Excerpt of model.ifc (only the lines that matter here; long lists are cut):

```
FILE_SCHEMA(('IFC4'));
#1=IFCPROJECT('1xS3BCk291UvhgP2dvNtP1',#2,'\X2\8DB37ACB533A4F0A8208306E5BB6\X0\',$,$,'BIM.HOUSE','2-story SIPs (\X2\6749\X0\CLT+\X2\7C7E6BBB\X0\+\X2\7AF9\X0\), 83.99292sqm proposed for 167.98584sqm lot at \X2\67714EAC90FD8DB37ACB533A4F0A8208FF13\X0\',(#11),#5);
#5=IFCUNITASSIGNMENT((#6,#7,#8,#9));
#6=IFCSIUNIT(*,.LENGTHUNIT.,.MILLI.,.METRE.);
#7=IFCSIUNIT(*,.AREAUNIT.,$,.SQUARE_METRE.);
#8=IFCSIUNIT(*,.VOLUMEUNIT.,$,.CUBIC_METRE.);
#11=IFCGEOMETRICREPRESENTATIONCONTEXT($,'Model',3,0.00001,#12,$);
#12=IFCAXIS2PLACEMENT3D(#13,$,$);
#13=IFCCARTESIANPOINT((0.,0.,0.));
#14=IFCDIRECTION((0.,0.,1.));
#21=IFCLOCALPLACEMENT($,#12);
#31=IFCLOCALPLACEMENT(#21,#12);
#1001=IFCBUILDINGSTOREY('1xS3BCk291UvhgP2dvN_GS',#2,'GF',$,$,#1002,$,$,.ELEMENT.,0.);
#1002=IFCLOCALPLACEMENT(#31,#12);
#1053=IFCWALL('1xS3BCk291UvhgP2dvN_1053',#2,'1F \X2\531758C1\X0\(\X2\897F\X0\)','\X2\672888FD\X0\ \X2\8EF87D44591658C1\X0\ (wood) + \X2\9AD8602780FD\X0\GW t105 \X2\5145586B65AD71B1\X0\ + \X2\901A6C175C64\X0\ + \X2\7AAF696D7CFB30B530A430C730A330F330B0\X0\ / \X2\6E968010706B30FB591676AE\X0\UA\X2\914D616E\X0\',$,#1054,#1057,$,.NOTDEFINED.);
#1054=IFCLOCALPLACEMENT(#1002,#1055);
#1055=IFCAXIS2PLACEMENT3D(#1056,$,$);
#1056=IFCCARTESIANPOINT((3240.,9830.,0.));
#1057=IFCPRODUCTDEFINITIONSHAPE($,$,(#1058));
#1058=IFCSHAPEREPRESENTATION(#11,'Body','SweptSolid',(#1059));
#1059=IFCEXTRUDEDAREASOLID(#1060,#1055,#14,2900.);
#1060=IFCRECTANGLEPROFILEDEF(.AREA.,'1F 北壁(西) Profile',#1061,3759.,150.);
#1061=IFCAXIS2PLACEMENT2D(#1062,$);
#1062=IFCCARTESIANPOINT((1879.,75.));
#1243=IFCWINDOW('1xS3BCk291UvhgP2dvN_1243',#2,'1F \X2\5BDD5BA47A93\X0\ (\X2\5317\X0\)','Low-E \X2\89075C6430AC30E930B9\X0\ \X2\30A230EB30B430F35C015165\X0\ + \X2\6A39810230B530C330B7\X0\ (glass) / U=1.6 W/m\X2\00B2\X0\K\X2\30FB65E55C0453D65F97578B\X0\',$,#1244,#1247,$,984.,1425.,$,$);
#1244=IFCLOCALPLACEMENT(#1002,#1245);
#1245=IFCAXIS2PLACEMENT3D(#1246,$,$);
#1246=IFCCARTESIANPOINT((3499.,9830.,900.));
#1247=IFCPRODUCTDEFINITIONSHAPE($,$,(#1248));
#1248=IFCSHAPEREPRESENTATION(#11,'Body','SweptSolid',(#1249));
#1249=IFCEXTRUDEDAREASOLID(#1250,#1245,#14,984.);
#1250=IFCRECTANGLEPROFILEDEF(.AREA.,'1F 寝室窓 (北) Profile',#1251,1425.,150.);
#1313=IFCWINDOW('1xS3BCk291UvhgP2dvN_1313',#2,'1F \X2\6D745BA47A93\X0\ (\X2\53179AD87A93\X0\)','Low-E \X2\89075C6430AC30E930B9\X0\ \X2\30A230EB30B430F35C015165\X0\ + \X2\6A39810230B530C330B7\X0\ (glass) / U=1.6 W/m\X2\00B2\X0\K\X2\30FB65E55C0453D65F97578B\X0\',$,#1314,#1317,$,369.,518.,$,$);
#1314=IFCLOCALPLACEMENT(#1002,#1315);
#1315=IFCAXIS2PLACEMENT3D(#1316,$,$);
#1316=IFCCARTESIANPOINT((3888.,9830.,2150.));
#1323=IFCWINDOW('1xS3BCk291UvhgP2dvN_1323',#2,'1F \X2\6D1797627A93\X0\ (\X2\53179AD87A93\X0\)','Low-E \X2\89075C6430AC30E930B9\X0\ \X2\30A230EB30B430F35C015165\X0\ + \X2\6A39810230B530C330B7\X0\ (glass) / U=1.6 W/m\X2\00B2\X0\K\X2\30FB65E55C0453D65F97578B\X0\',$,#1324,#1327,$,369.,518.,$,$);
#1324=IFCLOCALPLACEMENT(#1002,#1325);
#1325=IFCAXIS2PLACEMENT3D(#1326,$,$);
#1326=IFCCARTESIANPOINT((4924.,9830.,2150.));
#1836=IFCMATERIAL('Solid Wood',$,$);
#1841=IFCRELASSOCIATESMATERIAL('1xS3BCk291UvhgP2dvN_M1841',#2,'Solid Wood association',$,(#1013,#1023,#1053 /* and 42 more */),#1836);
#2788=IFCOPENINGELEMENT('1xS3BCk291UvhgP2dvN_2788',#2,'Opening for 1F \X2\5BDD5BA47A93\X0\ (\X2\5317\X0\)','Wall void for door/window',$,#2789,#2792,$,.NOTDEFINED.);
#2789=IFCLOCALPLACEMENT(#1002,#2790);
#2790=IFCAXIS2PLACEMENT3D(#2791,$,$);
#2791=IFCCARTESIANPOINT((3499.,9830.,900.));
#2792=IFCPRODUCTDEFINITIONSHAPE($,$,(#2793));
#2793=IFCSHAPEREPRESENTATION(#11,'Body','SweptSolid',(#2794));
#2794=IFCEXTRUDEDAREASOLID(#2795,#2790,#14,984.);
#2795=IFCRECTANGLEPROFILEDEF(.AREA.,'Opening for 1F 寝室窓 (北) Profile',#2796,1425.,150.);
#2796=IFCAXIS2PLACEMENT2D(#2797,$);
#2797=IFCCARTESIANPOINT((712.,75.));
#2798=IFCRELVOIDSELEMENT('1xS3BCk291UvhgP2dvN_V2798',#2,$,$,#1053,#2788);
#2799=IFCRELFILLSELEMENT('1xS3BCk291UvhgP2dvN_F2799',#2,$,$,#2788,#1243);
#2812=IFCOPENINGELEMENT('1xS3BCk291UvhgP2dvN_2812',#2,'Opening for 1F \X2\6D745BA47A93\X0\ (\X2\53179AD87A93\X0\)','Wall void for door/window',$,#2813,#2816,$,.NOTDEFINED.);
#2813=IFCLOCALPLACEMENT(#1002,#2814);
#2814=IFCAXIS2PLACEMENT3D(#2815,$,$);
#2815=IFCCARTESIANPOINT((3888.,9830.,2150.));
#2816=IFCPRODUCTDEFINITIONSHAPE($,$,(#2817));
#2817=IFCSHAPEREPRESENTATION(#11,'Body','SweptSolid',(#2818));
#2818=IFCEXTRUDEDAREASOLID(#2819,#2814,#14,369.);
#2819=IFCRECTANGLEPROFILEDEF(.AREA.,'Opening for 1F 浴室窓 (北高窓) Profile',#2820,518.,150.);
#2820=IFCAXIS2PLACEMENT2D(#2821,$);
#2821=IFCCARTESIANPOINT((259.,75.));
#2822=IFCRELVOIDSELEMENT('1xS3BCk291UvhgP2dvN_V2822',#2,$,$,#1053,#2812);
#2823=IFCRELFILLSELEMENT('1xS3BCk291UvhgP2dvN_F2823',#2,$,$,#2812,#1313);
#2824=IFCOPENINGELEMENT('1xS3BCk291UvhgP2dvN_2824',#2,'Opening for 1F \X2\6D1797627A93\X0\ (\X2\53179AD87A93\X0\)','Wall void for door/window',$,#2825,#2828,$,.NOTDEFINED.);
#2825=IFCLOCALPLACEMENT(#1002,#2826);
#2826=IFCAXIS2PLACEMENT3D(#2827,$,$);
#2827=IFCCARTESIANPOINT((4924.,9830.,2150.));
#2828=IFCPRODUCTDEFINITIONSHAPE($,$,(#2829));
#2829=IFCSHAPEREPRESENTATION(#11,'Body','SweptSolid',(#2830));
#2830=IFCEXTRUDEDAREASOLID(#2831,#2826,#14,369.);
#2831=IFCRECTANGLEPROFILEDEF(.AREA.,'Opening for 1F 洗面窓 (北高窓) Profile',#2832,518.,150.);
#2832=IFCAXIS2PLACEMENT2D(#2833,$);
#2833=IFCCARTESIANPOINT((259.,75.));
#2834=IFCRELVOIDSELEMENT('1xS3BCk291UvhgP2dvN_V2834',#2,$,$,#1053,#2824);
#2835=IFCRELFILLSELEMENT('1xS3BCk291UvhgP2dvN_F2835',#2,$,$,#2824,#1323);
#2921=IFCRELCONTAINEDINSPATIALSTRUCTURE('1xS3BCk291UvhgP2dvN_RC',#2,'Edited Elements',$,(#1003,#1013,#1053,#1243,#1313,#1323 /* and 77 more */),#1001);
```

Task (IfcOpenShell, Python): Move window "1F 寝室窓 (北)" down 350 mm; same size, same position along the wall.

```python
import numpy as np
import ifcopenshell
import ifcopenshell.api.geometry
import ifcopenshell.util.placement
import ifcopenshell.util.unit

model = ifcopenshell.open("model.ifc")
unit_scale = ifcopenshell.util.unit.calculate_unit_scale(model)

window = model.by_guid("1xS3BCk291UvhgP2dvN_1243")
opening = window.FillsVoids[0].RelatingOpeningElement
dz = -350.0

shift = np.array([0.0, 0.0, dz])
# The window is not placed relative to its opening, so move both.
for product in (opening, window):
    matrix = ifcopenshell.util.placement.get_local_placement(product.ObjectPlacement)
    matrix[:3, 3] += shift
    ifcopenshell.api.geometry.edit_object_placement(model, product=product, matrix=matrix, is_si=False)

print(f"moved by {dz * unit_scale:+.3f} m")

model.write("model-out.ifc")
```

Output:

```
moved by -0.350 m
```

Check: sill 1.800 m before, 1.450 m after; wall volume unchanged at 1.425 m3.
